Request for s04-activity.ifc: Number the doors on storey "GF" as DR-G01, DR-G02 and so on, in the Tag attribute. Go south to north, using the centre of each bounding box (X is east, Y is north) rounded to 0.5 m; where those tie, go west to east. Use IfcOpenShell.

First a look at what the model holds.

```python
import ifcopenshell
import ifcopenshell.util.element
import ifcopenshell.util.placement

model = ifcopenshell.open("s04-activity.ifc")
print(model.schema)
storey = next(s for s in model.by_type("IfcBuildingStorey") if s.Name == "GF")
doors = [e for e in ifcopenshell.util.element.get_decomposition(storey) if e.is_a("IfcDoor")]
for e in sorted(doors, key=lambda e: e.id()):
    origin = ifcopenshell.util.placement.get_local_placement(e.ObjectPlacement)[:3, 3]
    print(e.id(), e.Tag, e.Name, origin.round(2) + 0.0, sep=" | ")
```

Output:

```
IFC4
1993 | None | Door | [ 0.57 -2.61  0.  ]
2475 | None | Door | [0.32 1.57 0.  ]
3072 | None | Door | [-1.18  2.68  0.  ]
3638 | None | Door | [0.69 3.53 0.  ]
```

```python
import ifcopenshell
import ifcopenshell.geom
import ifcopenshell.util.element
import ifcopenshell.util.shape

model = ifcopenshell.open("s04-activity.ifc")
settings = ifcopenshell.geom.settings()
settings.set("use-world-coords", True)


def centre(element):
    shape = ifcopenshell.geom.create_shape(settings, element)
    return ifcopenshell.util.shape.get_bbox_centroid(shape.geometry)


storey = next(s for s in model.by_type("IfcBuildingStorey") if s.Name == "GF")
doors = [e for e in ifcopenshell.util.element.get_decomposition(storey) if e.is_a("IfcDoor")]

# Insertion points can sit at a corner or the storey origin, so sort by the geometry (in metres).
centres = {e: centre(e) for e in doors}
doors.sort(key=lambda e: (round(centres[e][1] / 0.5), centres[e][0]))

for i, e in enumerate(doors, start=1):
    number = f"DR-G{i:02d}"
    e.Tag = number
    print(e.id(), number)

model.write("s04-activity_updated.ifc")
```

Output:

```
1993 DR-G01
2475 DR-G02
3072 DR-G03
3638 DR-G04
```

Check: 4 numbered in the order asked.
